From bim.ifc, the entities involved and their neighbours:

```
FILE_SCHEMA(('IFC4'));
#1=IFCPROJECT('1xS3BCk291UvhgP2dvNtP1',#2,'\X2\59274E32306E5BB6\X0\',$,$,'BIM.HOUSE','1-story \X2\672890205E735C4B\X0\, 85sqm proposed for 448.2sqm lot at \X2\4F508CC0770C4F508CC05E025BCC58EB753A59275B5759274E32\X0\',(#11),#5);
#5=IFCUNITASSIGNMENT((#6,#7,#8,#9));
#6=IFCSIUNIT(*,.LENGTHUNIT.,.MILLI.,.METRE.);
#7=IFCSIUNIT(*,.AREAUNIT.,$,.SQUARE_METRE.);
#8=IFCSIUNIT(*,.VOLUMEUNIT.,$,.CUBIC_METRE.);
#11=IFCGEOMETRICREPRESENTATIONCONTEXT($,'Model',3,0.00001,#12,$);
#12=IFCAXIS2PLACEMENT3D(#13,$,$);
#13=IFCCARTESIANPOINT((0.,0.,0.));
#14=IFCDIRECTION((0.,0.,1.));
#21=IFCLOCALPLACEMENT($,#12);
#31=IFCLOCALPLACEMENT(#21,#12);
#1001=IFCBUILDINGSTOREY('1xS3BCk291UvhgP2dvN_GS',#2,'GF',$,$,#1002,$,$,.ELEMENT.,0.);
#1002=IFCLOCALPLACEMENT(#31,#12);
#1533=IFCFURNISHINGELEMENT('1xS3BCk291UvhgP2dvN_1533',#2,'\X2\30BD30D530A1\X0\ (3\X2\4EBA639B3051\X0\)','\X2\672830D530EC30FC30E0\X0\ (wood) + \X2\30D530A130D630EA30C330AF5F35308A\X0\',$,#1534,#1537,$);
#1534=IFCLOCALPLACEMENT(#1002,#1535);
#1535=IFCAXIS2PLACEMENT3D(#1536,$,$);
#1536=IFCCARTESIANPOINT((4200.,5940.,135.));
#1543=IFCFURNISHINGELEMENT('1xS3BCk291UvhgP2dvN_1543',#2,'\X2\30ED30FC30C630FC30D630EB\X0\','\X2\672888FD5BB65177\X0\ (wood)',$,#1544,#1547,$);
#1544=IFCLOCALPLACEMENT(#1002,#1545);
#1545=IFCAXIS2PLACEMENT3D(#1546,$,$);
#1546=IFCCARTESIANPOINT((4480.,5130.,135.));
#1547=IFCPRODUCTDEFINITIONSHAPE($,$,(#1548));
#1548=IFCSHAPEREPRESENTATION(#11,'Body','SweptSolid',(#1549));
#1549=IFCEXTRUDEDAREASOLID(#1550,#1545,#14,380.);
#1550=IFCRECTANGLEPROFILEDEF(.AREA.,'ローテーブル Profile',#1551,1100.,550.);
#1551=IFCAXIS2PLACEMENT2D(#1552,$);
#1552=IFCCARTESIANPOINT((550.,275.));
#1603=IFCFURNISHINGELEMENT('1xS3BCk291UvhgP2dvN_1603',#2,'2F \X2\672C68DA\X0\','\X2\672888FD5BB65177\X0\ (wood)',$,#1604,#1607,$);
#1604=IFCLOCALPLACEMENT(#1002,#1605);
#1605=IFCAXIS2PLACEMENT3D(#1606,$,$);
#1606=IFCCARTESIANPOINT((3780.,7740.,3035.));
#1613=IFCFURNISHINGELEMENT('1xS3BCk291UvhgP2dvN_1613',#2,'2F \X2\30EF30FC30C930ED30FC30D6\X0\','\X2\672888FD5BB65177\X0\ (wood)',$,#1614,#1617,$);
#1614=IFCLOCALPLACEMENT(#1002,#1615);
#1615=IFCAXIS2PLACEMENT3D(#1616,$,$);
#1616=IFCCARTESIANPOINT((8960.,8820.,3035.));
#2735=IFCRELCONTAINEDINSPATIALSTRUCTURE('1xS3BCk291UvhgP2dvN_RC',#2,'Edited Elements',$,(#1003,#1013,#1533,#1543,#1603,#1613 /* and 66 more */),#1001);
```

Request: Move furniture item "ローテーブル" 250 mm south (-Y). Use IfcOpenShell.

```python
import ifcopenshell
import ifcopenshell.api.geometry
import ifcopenshell.util.placement
import ifcopenshell.util.unit

model = ifcopenshell.open("bim.ifc")
unit_scale = ifcopenshell.util.unit.calculate_unit_scale(model)

item = model.by_guid("1xS3BCk291UvhgP2dvN_1543")
matrix = ifcopenshell.util.placement.get_local_placement(item.ObjectPlacement)
matrix[1, 3] -= 0.25 / unit_scale
ifcopenshell.api.geometry.edit_object_placement(model, product=item, matrix=matrix, is_si=False)

print(ifcopenshell.util.placement.get_local_placement(item.ObjectPlacement).round(3) + 0.0)

model.write("bim_updated.ifc")
```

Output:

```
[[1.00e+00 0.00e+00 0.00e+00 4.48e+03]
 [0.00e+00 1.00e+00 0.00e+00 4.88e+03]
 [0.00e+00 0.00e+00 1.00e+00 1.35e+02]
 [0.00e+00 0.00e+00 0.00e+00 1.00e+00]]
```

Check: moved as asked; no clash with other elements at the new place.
